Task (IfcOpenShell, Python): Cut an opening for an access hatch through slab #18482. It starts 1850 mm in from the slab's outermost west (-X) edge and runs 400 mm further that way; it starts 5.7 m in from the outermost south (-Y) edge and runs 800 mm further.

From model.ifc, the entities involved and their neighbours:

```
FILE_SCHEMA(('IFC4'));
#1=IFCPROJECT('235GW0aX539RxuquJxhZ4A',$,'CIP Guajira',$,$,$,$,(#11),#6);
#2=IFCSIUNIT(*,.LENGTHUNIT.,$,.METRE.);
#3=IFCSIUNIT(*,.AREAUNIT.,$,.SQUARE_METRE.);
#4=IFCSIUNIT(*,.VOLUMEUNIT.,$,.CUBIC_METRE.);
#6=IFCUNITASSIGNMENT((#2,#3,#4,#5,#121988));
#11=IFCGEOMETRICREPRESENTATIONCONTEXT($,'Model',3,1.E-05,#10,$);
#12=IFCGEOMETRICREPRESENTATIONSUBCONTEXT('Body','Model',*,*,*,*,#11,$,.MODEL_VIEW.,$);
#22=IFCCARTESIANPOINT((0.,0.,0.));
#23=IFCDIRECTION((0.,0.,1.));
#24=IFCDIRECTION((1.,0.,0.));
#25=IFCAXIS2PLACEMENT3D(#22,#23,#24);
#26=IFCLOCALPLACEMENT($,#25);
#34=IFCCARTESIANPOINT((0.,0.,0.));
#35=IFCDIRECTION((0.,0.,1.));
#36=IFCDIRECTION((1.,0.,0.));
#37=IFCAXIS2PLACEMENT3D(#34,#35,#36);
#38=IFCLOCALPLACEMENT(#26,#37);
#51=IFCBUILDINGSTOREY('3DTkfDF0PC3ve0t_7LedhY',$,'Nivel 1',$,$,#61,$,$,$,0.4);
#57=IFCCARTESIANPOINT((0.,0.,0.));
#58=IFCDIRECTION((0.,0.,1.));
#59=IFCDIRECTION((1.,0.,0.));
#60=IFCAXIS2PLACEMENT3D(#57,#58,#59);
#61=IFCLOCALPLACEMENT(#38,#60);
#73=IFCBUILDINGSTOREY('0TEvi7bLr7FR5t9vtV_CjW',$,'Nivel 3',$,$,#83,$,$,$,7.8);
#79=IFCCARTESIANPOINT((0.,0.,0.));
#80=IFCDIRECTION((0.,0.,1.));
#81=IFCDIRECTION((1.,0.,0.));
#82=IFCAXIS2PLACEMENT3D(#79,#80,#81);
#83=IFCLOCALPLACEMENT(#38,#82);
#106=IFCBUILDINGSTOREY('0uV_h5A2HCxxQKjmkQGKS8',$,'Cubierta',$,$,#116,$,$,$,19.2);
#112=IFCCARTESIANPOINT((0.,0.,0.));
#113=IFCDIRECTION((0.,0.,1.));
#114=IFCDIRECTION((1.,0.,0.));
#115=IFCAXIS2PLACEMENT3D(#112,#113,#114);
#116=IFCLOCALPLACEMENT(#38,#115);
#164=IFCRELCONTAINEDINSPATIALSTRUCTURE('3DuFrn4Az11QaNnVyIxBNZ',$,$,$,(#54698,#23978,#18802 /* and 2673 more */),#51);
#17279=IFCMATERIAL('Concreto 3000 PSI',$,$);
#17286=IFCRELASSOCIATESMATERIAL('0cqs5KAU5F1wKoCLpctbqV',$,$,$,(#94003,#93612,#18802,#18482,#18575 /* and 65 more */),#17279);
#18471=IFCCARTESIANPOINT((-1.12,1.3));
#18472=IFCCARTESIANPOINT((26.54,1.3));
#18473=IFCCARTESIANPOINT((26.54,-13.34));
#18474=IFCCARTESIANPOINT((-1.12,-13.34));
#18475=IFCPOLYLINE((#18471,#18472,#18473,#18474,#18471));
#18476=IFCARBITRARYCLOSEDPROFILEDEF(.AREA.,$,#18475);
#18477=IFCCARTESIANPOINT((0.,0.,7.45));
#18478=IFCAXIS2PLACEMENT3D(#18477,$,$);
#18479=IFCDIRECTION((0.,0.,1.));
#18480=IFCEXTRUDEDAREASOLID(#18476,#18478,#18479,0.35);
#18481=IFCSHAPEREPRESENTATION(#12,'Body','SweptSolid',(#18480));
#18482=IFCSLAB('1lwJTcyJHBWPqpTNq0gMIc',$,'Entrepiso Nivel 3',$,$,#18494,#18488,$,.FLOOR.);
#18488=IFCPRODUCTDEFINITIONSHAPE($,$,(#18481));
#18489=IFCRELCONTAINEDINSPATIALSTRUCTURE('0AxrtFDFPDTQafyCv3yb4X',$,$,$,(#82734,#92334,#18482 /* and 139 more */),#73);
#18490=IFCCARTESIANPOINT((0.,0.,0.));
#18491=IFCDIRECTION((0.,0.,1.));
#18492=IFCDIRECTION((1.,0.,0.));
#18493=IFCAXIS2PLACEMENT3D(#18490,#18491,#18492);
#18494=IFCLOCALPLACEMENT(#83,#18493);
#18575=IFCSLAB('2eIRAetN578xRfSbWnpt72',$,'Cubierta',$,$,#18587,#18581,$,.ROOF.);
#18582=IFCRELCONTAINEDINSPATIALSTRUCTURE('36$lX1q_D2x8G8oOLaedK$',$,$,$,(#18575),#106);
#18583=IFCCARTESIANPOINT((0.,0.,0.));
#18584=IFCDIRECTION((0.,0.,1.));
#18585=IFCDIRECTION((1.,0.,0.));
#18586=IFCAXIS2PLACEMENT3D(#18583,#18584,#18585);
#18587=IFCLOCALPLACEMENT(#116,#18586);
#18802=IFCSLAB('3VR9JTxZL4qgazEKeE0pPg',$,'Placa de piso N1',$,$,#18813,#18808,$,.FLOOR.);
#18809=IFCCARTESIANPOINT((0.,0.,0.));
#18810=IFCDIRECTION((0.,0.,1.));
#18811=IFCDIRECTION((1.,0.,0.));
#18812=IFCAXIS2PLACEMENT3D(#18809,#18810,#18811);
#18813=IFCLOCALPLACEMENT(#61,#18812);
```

```python
import numpy as np
import ifcopenshell
import ifcopenshell.api.feature
import ifcopenshell.api.geometry
import ifcopenshell.api.root
import ifcopenshell.geom
import ifcopenshell.util.placement
import ifcopenshell.util.representation
import ifcopenshell.util.shape
import ifcopenshell.util.unit

model = ifcopenshell.open("model.ifc")
unit_scale = ifcopenshell.util.unit.calculate_unit_scale(model)
settings = ifcopenshell.geom.settings()


def volume(element):
    """Net volume in cubic metres, openings subtracted."""
    shape = ifcopenshell.geom.create_shape(settings, element)
    return ifcopenshell.util.shape.get_volume(shape.geometry)


slab = model.by_guid("1lwJTcyJHBWPqpTNq0gMIc")
before = volume(slab)

# Extent in the slab's own axes, in metres. The edges named are its -X and -Y sides.
slab_shape = ifcopenshell.geom.create_shape(settings, slab)
vertices = ifcopenshell.util.shape.get_vertices(slab_shape.geometry)
x_min, y_min, bottom = vertices.min(axis=0)
top = vertices[:, 2].max()

opening = ifcopenshell.api.root.create_entity(model, ifc_class="IfcOpeningElement", name="Access hatch opening", predefined_type="OPENING")
context = ifcopenshell.util.representation.get_context(model, "Model", "Body", "MODEL_VIEW")
width, depth = 0.4, 0.8
outline = [(0.0, 0.0), (width, 0.0), (width, depth), (0.0, depth), (0.0, 0.0)]
# Overshoot both faces by 50 mm so the cut is clean.
shape = ifcopenshell.api.geometry.add_slab_representation(
    model, context=context, depth=top - bottom + 0.1, polyline=outline
)
ifcopenshell.api.geometry.assign_representation(model, product=opening, representation=shape)

matrix = ifcopenshell.util.placement.get_local_placement(slab.ObjectPlacement)
matrix[:, 3] = matrix @ np.append(np.array([x_min + 1.85, y_min + 5.7, bottom - 0.05]) / unit_scale, 1.0)
ifcopenshell.api.geometry.edit_object_placement(model, product=opening, matrix=matrix, is_si=False)
ifcopenshell.api.feature.add_feature(model, feature=opening, element=slab)

after = volume(slab)

print(f"slab volume {before:.3f} -> {after:.3f} m3")

model.write("model-out.ifc")
```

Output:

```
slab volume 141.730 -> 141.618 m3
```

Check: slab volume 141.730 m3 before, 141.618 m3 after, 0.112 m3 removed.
